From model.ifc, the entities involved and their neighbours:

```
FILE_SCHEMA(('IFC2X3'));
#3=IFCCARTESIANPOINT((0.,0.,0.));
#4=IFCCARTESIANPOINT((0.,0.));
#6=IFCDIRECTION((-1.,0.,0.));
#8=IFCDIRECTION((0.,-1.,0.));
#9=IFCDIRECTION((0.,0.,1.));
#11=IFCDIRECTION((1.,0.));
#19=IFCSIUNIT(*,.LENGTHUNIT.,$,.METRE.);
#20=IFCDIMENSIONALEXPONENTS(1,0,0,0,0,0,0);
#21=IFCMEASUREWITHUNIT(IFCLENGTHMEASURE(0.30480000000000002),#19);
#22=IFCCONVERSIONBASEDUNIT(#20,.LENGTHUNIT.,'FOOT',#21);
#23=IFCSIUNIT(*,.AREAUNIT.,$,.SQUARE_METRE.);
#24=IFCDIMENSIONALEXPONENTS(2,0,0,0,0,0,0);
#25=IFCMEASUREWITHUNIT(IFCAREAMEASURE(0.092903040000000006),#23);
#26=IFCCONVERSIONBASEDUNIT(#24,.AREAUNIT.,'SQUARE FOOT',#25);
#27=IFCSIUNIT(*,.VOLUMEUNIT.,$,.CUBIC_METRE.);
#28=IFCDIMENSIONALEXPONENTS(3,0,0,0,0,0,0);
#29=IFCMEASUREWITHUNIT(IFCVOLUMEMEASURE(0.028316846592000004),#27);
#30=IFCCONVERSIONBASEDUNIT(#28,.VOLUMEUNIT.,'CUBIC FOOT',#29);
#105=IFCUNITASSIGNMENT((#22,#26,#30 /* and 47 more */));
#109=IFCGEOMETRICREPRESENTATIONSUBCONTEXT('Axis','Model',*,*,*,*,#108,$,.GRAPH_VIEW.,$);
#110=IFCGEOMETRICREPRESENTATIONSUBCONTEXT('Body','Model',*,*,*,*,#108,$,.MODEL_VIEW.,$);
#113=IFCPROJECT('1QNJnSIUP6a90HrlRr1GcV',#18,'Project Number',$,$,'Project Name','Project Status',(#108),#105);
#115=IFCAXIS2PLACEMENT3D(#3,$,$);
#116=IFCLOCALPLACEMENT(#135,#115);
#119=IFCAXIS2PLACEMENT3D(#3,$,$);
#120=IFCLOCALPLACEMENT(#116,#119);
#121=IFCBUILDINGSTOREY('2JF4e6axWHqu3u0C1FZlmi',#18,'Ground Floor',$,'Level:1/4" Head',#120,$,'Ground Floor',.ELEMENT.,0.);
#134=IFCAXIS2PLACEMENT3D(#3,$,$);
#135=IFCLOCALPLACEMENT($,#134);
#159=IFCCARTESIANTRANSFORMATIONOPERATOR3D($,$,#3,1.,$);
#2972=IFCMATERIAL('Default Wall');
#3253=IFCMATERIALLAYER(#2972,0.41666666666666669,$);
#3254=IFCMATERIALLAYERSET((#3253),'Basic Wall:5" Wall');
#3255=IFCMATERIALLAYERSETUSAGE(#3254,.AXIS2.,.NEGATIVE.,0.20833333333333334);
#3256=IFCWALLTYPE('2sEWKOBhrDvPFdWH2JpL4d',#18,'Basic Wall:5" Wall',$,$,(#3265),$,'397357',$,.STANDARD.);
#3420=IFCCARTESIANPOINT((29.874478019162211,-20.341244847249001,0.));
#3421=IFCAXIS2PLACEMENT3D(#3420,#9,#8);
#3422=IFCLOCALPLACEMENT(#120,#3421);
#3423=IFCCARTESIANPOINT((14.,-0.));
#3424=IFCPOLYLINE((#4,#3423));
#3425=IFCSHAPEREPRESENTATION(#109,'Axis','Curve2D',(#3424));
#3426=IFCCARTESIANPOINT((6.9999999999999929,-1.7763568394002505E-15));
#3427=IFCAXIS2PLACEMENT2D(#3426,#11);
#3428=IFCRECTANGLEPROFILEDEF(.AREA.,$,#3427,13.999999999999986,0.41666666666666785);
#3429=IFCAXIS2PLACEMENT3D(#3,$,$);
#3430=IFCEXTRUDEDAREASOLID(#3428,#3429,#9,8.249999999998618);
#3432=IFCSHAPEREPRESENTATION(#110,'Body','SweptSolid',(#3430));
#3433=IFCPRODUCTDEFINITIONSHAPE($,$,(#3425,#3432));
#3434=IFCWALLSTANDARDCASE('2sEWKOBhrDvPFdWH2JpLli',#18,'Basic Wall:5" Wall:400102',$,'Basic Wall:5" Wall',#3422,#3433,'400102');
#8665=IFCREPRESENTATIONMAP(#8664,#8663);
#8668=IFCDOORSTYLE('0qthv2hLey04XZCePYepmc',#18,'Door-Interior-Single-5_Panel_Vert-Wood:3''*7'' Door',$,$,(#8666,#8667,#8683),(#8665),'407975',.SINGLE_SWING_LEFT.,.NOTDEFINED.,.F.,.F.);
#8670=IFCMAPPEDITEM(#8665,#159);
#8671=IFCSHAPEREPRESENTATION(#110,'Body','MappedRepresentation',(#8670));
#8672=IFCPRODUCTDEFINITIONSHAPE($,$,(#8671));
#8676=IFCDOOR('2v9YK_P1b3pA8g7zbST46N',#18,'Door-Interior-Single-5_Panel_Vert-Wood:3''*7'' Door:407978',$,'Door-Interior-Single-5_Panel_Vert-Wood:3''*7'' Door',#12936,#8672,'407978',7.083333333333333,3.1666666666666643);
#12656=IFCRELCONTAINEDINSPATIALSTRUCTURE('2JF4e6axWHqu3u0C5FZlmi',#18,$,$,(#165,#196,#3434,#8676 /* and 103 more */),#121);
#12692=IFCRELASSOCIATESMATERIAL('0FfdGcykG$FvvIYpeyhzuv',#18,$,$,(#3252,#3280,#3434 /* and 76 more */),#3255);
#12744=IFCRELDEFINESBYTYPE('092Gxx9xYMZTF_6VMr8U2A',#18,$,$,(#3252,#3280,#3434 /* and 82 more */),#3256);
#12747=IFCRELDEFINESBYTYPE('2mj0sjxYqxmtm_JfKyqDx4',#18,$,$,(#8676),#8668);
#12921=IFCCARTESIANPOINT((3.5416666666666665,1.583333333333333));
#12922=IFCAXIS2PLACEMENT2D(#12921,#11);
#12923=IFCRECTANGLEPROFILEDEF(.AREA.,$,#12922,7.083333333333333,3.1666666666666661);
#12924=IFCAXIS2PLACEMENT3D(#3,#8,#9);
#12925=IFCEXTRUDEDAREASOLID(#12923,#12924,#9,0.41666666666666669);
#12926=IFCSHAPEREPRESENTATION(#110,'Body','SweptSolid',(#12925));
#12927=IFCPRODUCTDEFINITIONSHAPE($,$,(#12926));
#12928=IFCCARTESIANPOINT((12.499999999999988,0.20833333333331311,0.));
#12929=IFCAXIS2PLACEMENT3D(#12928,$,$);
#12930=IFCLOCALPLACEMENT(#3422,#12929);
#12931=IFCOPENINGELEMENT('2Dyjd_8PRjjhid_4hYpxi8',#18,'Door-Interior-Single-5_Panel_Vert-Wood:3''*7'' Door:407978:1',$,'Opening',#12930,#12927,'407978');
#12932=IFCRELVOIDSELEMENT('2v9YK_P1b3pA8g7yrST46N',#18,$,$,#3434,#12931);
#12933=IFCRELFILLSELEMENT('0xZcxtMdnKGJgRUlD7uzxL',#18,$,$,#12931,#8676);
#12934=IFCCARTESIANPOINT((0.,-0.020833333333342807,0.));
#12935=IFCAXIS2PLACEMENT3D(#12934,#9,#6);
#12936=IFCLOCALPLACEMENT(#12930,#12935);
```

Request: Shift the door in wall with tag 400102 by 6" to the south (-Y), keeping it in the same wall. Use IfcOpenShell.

```python
import ifcopenshell
import ifcopenshell.api.geometry
import ifcopenshell.util.placement
import ifcopenshell.util.unit

model = ifcopenshell.open("model.ifc")
unit_scale = ifcopenshell.util.unit.calculate_unit_scale(model)

door = model.by_guid("2v9YK_P1b3pA8g7zbST46N")
opening = door.FillsVoids[0].RelatingOpeningElement
wall = opening.VoidsElements[0].RelatingBuildingElement

wall_matrix = ifcopenshell.util.placement.get_local_placement(wall.ObjectPlacement)
shift = wall_matrix[:3, 0] * 6 * 0.0254 / unit_scale
before = ifcopenshell.util.placement.get_local_placement(door.ObjectPlacement)[:3, 3].copy()

# The door is placed relative to its opening, so it follows when the opening moves.
matrix = ifcopenshell.util.placement.get_local_placement(opening.ObjectPlacement)
matrix[:3, 3] += shift
ifcopenshell.api.geometry.edit_object_placement(
    model, product=opening, matrix=matrix, is_si=False, should_transform_children=True
)

after = ifcopenshell.util.placement.get_local_placement(door.ObjectPlacement)[:3, 3]
print("door moved by", (after - before).round(3) + 0.0)

model.write("model_edited.ifc")
```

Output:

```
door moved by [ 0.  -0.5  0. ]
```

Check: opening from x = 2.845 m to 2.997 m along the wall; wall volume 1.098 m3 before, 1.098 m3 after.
